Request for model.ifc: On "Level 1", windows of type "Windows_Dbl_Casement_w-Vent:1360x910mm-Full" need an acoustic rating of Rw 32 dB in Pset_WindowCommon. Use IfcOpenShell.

First a look at what the model holds.

```python
import ifcopenshell
import ifcopenshell.util.element

model = ifcopenshell.open("model.ifc")
print(model.schema)
storey = next(s for s in model.by_type("IfcBuildingStorey") if s.Name == "Level 1")
windows = [e for e in ifcopenshell.util.element.get_decomposition(storey) if e.is_a("IfcWindow")]
seen = {}
for e in windows:
    element_type = ifcopenshell.util.element.get_type(e)
    key = (element_type.Name if element_type != e and element_type else None, ifcopenshell.util.element.get_pset(e, "Pset_WindowCommon", "AcousticRating"))
    seen[key] = seen.get(key, 0) + 1
for (name, value), count in sorted(seen.items(), key=str):
    print(count, "x", name, "|", value)
```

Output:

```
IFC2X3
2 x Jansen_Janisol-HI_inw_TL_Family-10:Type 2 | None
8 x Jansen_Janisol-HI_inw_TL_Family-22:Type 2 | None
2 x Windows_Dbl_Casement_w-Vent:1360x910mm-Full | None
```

```python
import ifcopenshell
import ifcopenshell.api.pset
import ifcopenshell.util.element

model = ifcopenshell.open("model.ifc")

storey = next(s for s in model.by_type("IfcBuildingStorey") if s.Name == "Level 1")
windows = [e for e in ifcopenshell.util.element.get_decomposition(storey) if e.is_a("IfcWindow")]

count = 0
for e in windows:
    element_type = ifcopenshell.util.element.get_type(e)
    if element_type in (None, e) or element_type.Name != "Windows_Dbl_Casement_w-Vent:1360x910mm-Full":
        continue
    # add_pset returns the element's existing set when there is one.
    pset = ifcopenshell.api.pset.add_pset(model, product=e, name="Pset_WindowCommon")
    ifcopenshell.api.pset.edit_pset(model, pset=pset, properties={"AcousticRating": "Rw 32 dB"})
    count += 1

print(count, "windows updated")

model.write("model_updated.ifc")
```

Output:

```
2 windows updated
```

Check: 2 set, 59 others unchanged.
